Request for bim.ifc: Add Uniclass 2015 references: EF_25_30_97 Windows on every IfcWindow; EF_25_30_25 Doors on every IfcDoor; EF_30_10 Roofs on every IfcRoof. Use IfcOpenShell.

First a look at what the model holds.

```python
import ifcopenshell

model = ifcopenshell.open("bim.ifc")
print(model.schema)
print("classifications:", [c.Name for c in model.by_type("IfcClassification")])
for ifc_class in ("IfcDoor", "IfcRoof", "IfcStair", "IfcWall", "IfcWindow"):
    print(ifc_class, len(model.by_type(ifc_class)))
```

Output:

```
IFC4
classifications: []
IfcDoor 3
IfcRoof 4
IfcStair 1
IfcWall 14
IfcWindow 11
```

```python
import ifcopenshell
import ifcopenshell.api.classification

model = ifcopenshell.open("bim.ifc")

system = ifcopenshell.api.classification.add_classification(model, classification="Uniclass 2015")

codes = {
    "IfcWindow": ("EF_25_30_97", "Windows"),
    "IfcDoor": ("EF_25_30_25", "Doors"),
    "IfcRoof": ("EF_30_10", "Roofs"),
}
for ifc_class, (code, name) in codes.items():
    products = model.by_type(ifc_class)
    ifcopenshell.api.classification.add_reference(
        model, products=products, classification=system, identification=code, name=name
    )
    print(code, len(products))

model.write("bim_rev.ifc")
```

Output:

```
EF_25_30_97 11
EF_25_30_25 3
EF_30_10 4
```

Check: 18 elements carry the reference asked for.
